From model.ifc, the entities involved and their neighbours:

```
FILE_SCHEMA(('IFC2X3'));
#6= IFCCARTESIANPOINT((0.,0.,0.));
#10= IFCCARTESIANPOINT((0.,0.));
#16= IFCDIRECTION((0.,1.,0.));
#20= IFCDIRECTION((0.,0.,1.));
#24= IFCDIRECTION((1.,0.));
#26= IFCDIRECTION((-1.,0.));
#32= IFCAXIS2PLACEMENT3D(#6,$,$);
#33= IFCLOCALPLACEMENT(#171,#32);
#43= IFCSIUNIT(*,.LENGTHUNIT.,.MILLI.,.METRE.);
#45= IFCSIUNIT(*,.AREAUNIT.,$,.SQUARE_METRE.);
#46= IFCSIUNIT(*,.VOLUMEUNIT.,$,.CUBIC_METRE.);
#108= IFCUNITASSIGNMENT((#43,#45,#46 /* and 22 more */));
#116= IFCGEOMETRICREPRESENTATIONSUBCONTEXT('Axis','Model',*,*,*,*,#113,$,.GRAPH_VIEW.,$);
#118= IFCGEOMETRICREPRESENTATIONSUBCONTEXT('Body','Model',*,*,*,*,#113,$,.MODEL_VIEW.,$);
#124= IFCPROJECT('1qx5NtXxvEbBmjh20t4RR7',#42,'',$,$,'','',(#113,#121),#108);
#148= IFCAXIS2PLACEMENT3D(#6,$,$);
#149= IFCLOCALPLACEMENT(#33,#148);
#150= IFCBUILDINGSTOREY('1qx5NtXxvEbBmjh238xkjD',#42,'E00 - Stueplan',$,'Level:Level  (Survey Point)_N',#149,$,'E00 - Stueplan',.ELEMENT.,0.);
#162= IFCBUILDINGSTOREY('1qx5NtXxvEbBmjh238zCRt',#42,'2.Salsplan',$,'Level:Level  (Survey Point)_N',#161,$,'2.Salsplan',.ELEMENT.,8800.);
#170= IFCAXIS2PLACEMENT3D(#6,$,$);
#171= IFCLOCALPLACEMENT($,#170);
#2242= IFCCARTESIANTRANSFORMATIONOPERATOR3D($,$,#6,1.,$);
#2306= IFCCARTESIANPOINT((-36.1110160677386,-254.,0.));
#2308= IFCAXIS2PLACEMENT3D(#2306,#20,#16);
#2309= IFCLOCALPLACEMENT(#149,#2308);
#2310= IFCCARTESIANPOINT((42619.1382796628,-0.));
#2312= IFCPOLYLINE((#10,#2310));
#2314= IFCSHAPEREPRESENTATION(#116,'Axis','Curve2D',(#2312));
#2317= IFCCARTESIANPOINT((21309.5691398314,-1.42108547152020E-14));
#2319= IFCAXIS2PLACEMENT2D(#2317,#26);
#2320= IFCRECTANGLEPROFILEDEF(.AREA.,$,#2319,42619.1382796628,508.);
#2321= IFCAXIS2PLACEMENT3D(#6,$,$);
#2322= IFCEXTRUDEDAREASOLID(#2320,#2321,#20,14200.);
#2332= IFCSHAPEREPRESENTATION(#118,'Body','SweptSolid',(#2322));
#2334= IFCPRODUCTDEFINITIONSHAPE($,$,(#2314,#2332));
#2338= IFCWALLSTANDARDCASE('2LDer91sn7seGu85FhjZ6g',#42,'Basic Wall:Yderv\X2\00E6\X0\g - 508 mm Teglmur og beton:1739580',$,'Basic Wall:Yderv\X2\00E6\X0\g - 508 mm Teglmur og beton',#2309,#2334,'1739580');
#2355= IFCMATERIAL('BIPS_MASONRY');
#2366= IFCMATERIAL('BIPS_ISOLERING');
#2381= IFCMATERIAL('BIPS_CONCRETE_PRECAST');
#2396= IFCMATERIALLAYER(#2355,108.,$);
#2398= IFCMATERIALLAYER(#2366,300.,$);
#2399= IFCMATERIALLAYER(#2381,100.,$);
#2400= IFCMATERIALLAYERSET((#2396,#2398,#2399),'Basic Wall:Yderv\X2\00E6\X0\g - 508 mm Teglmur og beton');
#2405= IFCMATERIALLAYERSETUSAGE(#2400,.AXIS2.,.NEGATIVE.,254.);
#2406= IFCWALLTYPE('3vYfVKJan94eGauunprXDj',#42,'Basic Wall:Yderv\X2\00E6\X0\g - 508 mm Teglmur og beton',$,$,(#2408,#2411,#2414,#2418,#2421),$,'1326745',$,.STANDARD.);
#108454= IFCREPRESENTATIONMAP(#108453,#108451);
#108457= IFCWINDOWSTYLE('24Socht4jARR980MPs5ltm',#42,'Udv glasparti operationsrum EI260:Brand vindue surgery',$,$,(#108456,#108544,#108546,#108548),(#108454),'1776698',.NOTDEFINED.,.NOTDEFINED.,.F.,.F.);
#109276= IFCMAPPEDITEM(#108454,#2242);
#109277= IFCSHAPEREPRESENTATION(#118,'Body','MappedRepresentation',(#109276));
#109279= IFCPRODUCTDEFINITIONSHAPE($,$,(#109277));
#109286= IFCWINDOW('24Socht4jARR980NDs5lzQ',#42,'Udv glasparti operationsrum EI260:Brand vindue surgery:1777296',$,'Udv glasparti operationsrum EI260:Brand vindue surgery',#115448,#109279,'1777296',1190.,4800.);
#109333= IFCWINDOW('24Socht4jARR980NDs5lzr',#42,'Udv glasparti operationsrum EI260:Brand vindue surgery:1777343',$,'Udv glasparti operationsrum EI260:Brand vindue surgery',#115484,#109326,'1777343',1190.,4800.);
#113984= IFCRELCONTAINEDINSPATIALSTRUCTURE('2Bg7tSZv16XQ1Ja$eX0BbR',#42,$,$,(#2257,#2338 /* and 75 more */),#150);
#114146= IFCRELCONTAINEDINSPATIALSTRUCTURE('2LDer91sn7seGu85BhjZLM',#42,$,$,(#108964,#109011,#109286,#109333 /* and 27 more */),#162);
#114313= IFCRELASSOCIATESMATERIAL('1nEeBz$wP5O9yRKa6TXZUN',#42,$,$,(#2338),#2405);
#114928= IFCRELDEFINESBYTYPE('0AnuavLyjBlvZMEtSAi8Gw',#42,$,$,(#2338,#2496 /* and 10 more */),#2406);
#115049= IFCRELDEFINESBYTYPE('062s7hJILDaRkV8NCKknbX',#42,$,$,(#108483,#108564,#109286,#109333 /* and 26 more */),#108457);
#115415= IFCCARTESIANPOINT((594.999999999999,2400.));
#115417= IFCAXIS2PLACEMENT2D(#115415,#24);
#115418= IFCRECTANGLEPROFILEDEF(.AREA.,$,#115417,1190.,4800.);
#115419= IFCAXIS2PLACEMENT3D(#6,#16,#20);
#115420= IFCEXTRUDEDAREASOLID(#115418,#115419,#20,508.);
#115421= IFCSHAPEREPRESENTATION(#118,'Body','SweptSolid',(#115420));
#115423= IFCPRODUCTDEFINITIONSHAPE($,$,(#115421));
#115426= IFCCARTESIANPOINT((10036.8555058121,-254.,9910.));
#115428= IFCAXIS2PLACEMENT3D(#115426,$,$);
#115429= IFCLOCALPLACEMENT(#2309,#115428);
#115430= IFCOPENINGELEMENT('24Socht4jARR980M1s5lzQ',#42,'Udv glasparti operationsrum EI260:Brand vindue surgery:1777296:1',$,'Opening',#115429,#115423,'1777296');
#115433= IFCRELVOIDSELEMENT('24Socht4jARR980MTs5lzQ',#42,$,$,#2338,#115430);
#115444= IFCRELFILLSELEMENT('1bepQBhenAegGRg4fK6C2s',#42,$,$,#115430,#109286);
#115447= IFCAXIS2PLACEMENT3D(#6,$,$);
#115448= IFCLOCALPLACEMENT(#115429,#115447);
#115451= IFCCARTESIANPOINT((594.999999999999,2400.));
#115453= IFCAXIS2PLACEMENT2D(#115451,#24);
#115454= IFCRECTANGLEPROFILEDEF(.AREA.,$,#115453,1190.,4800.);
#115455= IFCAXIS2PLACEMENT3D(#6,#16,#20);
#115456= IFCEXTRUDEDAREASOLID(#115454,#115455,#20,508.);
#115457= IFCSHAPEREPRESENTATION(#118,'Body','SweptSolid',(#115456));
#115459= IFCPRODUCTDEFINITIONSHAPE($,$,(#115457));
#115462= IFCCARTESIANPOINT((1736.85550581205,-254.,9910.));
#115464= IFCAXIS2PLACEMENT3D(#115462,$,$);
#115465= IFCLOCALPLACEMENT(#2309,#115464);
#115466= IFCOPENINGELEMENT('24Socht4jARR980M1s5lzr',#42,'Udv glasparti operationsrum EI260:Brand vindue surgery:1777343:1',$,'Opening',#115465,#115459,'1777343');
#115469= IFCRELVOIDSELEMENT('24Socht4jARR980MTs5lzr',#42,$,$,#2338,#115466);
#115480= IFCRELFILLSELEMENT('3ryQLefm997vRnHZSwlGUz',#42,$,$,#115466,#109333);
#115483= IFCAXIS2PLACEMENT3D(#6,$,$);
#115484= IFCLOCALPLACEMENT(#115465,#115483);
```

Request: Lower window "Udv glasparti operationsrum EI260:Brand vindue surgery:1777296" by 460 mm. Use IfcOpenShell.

```python
import numpy as np
import ifcopenshell
import ifcopenshell.api.geometry
import ifcopenshell.util.placement
import ifcopenshell.util.unit

model = ifcopenshell.open("model.ifc")
unit_scale = ifcopenshell.util.unit.calculate_unit_scale(model)

window = model.by_guid("24Socht4jARR980NDs5lzQ")
opening = window.FillsVoids[0].RelatingOpeningElement
dz = -460.0

shift = np.array([0.0, 0.0, dz])
# The window is placed relative to its opening, so it follows when the opening moves.
matrix = ifcopenshell.util.placement.get_local_placement(opening.ObjectPlacement)
matrix[:3, 3] += shift
ifcopenshell.api.geometry.edit_object_placement(
    model, product=opening, matrix=matrix, is_si=False, should_transform_children=True
)

print(f"moved by {dz * unit_scale:+.3f} m")

model.write("model_rev.ifc")
```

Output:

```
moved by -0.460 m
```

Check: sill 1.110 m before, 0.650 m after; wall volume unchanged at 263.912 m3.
